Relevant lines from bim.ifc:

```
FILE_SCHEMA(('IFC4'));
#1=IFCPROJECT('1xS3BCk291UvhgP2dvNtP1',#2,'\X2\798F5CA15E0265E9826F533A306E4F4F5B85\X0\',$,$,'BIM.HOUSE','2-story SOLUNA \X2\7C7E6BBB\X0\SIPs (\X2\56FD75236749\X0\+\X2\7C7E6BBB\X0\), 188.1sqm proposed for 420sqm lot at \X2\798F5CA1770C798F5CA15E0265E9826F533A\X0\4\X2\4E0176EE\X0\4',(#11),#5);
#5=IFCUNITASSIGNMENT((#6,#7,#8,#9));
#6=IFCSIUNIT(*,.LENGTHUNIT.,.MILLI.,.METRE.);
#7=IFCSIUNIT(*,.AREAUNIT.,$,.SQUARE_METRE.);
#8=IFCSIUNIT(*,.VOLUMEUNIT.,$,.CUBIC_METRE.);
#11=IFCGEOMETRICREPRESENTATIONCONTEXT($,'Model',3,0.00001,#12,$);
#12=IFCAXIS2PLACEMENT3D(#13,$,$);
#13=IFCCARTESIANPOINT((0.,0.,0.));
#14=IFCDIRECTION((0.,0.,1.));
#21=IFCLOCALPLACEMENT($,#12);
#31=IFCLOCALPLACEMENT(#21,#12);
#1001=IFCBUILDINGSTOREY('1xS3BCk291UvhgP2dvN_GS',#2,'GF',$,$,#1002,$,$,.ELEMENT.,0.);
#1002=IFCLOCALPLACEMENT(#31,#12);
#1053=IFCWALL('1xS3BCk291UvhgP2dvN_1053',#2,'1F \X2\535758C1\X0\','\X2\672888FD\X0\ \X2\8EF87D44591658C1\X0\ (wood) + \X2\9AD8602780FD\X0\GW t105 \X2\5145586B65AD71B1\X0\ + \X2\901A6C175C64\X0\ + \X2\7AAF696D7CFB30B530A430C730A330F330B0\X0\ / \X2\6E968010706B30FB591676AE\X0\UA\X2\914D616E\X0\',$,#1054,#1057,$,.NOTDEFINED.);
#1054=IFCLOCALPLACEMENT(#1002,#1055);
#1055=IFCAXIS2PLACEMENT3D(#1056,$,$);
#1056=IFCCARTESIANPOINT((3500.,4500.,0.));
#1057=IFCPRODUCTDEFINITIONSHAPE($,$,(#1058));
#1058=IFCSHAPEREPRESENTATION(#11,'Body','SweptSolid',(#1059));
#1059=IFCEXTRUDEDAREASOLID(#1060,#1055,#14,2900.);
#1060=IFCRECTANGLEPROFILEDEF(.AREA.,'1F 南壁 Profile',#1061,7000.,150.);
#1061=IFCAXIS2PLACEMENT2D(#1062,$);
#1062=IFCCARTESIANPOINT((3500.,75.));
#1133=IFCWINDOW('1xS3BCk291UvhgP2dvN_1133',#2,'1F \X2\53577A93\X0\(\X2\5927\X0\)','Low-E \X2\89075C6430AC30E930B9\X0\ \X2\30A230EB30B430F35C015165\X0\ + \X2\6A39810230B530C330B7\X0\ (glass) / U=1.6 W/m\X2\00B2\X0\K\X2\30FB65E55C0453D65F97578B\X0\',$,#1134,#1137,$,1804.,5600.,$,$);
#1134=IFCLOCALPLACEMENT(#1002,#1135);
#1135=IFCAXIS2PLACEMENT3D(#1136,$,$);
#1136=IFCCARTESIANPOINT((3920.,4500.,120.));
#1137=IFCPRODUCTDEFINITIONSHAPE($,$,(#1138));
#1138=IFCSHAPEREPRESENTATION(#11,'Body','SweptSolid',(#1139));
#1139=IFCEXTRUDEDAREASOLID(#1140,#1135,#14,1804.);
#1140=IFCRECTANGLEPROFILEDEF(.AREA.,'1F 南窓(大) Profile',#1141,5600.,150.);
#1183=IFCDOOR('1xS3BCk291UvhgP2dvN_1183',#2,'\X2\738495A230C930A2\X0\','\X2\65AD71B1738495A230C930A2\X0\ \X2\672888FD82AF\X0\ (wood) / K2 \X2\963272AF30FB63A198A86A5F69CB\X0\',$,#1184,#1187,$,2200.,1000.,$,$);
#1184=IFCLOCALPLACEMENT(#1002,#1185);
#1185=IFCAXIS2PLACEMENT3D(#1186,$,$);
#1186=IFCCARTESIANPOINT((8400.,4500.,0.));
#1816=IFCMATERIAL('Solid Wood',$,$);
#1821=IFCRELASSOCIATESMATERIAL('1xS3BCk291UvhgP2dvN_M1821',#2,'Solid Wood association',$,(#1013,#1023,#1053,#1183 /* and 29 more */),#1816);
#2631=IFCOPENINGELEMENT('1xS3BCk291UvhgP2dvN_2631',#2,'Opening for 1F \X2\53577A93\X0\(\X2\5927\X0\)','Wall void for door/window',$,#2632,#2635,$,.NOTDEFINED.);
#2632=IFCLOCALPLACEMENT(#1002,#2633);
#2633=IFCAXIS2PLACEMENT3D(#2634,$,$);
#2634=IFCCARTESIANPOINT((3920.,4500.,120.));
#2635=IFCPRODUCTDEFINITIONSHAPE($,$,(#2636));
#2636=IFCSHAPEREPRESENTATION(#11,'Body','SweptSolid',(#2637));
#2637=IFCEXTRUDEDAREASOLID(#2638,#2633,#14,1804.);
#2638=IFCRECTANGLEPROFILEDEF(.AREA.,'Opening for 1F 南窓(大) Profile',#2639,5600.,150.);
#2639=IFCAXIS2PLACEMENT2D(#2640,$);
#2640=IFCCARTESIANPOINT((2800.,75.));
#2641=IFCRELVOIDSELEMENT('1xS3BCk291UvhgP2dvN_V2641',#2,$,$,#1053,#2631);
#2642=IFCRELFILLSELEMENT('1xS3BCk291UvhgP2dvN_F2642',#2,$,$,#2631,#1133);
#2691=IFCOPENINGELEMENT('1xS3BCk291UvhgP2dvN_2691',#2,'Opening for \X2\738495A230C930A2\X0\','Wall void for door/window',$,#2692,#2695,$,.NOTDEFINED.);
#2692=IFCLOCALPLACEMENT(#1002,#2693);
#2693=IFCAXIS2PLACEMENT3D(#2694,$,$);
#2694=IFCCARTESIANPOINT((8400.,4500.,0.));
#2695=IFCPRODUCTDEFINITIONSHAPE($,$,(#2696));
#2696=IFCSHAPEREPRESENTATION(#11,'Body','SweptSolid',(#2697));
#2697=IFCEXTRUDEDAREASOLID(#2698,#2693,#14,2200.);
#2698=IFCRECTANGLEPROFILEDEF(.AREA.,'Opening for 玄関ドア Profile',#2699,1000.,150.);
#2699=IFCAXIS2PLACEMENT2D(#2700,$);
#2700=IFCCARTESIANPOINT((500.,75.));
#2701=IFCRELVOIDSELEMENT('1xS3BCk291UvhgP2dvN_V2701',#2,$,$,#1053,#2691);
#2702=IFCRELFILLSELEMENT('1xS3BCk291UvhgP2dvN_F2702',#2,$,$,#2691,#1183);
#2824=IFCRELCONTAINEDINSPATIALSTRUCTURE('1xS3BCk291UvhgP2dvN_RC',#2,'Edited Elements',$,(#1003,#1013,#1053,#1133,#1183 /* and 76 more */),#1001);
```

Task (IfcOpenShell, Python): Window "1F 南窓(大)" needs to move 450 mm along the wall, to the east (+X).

```python
import ifcopenshell
import ifcopenshell.api.geometry
import ifcopenshell.util.placement
import ifcopenshell.util.unit

model = ifcopenshell.open("bim.ifc")
unit_scale = ifcopenshell.util.unit.calculate_unit_scale(model)

window = model.by_id(1133)
opening = window.FillsVoids[0].RelatingOpeningElement
wall = opening.VoidsElements[0].RelatingBuildingElement

wall_matrix = ifcopenshell.util.placement.get_local_placement(wall.ObjectPlacement)
shift = wall_matrix[:3, 0] * 0.45 / unit_scale
before = ifcopenshell.util.placement.get_local_placement(window.ObjectPlacement)[:3, 3].copy()

# The window is not placed relative to its opening, so move both.
for product in (opening, window):
    matrix = ifcopenshell.util.placement.get_local_placement(product.ObjectPlacement)
    matrix[:3, 3] += shift
    ifcopenshell.api.geometry.edit_object_placement(model, product=product, matrix=matrix, is_si=False)

after = ifcopenshell.util.placement.get_local_placement(window.ObjectPlacement)[:3, 3]
print("window moved by", (after - before).round(3) + 0.0)

model.write("bim_edited.ifc")
```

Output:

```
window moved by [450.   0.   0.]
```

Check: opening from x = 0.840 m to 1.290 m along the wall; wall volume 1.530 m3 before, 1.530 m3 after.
